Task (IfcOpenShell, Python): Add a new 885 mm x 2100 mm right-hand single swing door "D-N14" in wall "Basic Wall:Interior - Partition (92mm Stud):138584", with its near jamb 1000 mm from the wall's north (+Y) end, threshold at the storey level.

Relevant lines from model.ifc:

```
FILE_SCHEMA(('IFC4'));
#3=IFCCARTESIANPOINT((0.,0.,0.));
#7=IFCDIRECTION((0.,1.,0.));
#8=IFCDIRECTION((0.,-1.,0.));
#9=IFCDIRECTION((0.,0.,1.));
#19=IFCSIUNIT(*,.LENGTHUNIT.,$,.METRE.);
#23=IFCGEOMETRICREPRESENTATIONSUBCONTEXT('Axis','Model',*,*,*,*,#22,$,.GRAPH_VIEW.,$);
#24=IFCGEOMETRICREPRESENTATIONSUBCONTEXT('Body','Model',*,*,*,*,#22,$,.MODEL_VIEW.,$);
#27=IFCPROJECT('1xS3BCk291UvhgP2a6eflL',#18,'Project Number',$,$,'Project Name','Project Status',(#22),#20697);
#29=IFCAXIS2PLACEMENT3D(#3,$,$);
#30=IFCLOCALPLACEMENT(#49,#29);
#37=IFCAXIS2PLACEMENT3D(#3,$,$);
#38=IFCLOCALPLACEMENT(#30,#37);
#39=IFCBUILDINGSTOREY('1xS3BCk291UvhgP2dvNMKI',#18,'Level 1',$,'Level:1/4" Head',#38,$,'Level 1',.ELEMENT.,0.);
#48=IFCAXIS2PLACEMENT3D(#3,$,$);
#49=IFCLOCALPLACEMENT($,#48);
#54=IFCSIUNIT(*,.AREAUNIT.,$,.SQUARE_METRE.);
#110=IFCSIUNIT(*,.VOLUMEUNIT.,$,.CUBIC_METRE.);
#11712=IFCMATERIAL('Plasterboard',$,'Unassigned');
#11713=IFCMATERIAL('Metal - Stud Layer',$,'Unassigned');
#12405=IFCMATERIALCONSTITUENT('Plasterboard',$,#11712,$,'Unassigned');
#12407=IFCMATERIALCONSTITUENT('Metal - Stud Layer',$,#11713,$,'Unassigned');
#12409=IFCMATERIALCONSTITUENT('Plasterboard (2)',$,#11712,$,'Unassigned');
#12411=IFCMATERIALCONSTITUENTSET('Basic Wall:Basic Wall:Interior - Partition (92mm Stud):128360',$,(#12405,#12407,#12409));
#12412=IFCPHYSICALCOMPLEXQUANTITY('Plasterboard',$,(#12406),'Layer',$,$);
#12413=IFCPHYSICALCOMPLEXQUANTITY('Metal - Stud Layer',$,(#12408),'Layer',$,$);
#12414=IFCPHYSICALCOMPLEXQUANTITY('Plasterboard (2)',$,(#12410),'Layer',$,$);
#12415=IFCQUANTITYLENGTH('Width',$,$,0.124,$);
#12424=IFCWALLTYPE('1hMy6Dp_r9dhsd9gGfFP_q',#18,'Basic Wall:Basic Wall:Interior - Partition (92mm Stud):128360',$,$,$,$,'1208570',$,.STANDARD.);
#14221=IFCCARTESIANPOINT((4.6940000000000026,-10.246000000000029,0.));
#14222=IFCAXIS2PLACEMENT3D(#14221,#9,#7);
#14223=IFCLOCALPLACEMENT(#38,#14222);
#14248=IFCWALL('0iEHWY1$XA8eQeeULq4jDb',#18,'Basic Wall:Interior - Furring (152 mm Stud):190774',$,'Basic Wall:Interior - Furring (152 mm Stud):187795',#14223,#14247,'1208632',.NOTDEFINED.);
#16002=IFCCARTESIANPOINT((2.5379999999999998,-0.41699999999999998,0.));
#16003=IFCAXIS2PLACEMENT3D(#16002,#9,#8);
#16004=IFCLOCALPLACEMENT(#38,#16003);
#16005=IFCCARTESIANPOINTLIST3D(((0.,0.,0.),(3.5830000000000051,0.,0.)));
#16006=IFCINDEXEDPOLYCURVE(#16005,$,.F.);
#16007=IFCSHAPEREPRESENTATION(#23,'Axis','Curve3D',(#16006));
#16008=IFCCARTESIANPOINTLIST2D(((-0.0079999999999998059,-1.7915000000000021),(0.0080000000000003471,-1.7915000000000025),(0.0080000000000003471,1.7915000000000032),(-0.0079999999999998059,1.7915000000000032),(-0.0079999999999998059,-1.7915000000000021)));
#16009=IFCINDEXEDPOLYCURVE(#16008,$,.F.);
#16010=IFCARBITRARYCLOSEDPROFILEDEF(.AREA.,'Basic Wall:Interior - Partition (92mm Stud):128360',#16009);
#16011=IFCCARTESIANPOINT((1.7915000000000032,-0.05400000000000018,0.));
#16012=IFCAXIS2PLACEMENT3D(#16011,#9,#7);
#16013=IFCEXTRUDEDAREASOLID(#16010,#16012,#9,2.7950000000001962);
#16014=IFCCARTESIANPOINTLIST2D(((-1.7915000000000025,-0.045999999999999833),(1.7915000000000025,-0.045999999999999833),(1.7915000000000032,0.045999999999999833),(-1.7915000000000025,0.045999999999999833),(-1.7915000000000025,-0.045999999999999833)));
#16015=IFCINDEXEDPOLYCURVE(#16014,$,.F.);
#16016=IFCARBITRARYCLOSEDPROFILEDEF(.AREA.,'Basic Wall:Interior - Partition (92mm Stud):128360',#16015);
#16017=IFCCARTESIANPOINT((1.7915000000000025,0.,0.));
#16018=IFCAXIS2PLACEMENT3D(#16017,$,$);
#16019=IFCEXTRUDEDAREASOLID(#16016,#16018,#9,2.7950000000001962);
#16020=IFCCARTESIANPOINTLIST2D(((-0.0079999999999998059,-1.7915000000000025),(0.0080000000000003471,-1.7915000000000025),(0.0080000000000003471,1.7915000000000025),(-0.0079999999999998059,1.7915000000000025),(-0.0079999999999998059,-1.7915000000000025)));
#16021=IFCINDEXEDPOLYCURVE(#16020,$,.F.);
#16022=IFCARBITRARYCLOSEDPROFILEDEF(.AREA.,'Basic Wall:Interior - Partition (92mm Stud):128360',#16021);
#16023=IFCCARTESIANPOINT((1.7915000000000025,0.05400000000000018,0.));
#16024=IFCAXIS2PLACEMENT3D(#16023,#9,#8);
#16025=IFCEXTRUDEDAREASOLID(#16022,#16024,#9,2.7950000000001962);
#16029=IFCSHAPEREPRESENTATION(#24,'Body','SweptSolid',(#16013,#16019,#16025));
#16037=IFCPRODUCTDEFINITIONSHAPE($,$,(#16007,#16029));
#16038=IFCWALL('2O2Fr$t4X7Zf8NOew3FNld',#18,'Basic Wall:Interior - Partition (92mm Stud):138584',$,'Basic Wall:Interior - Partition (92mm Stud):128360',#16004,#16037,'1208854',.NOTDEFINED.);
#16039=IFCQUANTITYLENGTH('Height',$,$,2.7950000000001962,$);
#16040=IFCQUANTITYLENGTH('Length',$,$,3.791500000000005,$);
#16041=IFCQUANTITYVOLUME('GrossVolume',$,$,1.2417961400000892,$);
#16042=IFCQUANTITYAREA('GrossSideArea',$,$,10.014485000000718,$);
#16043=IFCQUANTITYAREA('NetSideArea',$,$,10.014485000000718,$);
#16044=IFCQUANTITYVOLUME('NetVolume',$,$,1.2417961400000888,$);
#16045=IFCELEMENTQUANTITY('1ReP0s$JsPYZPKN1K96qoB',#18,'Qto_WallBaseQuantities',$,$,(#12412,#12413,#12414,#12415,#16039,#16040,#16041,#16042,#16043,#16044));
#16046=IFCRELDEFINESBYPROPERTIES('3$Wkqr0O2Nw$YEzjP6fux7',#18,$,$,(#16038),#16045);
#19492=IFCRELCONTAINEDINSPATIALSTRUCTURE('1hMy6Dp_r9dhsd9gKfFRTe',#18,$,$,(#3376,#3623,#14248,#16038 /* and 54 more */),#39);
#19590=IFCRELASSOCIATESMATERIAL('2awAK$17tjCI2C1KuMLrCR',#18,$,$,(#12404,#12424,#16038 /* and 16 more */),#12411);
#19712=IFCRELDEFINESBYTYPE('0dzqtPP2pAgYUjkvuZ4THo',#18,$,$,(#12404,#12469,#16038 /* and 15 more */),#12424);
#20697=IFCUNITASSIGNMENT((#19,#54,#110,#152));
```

```python
import numpy as np
import ifcopenshell
import ifcopenshell.api.feature
import ifcopenshell.api.geometry
import ifcopenshell.api.pset
import ifcopenshell.api.root
import ifcopenshell.api.spatial
import ifcopenshell.geom
import ifcopenshell.util.element
import ifcopenshell.util.placement
import ifcopenshell.util.representation
import ifcopenshell.util.shape
import ifcopenshell.util.unit

model = ifcopenshell.open("model.ifc")
unit_scale = ifcopenshell.util.unit.calculate_unit_scale(model)
area_scale = ifcopenshell.util.unit.calculate_unit_scale(model, "AREAUNIT")
volume_scale = ifcopenshell.util.unit.calculate_unit_scale(model, "VOLUMEUNIT")
settings = ifcopenshell.geom.settings()


def volume(element):
    """Net volume in cubic metres, openings subtracted."""
    shape = ifcopenshell.geom.create_shape(settings, element)
    return ifcopenshell.util.shape.get_volume(shape.geometry)


wall = model.by_guid("2O2Fr$t4X7Zf8NOew3FNld")
storey = ifcopenshell.util.element.get_container(wall, ifc_class="IfcBuildingStorey")
context = ifcopenshell.util.representation.get_context(model, "Model", "Body", "MODEL_VIEW")
before = volume(wall)

width, height, from_end, sill = 0.885, 2.1, 1, 0.0  # metres

# The wall runs along its own X axis, and the end named is its -X end.
wall_shape = ifcopenshell.geom.create_shape(settings, wall)
x, y, z = ifcopenshell.util.shape.get_vertices(wall_shape.geometry).T
start = x.min() + from_end
face, thickness = float(y.min()), float(y.max() - y.min())
wall_matrix = ifcopenshell.util.placement.get_local_placement(wall.ObjectPlacement)
level = ifcopenshell.util.placement.get_local_placement(storey.ObjectPlacement)[2, 3]


def in_wall(x, y):
    """Placement at x, y metres in the wall's axes, at sill height."""
    matrix = wall_matrix.copy()
    matrix[:, 3] = wall_matrix @ np.array([x / unit_scale, y / unit_scale, 0.0, 1.0])
    matrix[2, 3] = level + sill / unit_scale
    return matrix


# Opening: a box that overshoots both wall faces by 50 mm.
opening = ifcopenshell.api.root.create_entity(model, ifc_class="IfcOpeningElement", predefined_type="OPENING")
box = ifcopenshell.api.geometry.add_wall_representation(
    model, context=context, length=width, height=height, thickness=thickness + 0.1
)
ifcopenshell.api.geometry.assign_representation(model, product=opening, representation=box)
ifcopenshell.api.geometry.edit_object_placement(model, product=opening, matrix=in_wall(start, face - 0.05), is_si=False)
ifcopenshell.api.feature.add_feature(model, feature=opening, element=wall)

door = ifcopenshell.api.root.create_entity(model, ifc_class="IfcDoor", name="D-N14", predefined_type="DOOR")
door.OverallWidth, door.OverallHeight = width / unit_scale, height / unit_scale
door.OperationType = "SINGLE_SWING_RIGHT"
body = ifcopenshell.api.geometry.add_door_representation(
    model,
    context=context,
    overall_width=door.OverallWidth,
    overall_height=door.OverallHeight,
    operation_type="SINGLE_SWING_RIGHT",
    lining_properties={"LiningDepth": thickness / unit_scale, "ThresholdDepth": thickness / unit_scale},
)
ifcopenshell.api.geometry.assign_representation(model, product=door, representation=body)
ifcopenshell.api.spatial.assign_container(model, products=[door], relating_structure=storey)
ifcopenshell.api.feature.add_filling(model, opening=opening, element=door)

# The lining spans the wall, so the door starts at the wall face.
ifcopenshell.api.geometry.edit_object_placement(model, product=door, matrix=in_wall(start, face), is_si=False)

after = volume(wall)

# Update the wall's stored quantities.
qto = model.by_id(ifcopenshell.util.element.get_pset(wall, "Qto_WallBaseQuantities", should_inherit=False)["id"])
ifcopenshell.api.pset.edit_qto(model, qto=qto, properties={
    "NetSideArea": after / thickness / area_scale,
    "NetVolume": after / volume_scale,
})

print(f"wall volume {before:.3f} -> {after:.3f} m3")

model.write("model_edited.ifc")
```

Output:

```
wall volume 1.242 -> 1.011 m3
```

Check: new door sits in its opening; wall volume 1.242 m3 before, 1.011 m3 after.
